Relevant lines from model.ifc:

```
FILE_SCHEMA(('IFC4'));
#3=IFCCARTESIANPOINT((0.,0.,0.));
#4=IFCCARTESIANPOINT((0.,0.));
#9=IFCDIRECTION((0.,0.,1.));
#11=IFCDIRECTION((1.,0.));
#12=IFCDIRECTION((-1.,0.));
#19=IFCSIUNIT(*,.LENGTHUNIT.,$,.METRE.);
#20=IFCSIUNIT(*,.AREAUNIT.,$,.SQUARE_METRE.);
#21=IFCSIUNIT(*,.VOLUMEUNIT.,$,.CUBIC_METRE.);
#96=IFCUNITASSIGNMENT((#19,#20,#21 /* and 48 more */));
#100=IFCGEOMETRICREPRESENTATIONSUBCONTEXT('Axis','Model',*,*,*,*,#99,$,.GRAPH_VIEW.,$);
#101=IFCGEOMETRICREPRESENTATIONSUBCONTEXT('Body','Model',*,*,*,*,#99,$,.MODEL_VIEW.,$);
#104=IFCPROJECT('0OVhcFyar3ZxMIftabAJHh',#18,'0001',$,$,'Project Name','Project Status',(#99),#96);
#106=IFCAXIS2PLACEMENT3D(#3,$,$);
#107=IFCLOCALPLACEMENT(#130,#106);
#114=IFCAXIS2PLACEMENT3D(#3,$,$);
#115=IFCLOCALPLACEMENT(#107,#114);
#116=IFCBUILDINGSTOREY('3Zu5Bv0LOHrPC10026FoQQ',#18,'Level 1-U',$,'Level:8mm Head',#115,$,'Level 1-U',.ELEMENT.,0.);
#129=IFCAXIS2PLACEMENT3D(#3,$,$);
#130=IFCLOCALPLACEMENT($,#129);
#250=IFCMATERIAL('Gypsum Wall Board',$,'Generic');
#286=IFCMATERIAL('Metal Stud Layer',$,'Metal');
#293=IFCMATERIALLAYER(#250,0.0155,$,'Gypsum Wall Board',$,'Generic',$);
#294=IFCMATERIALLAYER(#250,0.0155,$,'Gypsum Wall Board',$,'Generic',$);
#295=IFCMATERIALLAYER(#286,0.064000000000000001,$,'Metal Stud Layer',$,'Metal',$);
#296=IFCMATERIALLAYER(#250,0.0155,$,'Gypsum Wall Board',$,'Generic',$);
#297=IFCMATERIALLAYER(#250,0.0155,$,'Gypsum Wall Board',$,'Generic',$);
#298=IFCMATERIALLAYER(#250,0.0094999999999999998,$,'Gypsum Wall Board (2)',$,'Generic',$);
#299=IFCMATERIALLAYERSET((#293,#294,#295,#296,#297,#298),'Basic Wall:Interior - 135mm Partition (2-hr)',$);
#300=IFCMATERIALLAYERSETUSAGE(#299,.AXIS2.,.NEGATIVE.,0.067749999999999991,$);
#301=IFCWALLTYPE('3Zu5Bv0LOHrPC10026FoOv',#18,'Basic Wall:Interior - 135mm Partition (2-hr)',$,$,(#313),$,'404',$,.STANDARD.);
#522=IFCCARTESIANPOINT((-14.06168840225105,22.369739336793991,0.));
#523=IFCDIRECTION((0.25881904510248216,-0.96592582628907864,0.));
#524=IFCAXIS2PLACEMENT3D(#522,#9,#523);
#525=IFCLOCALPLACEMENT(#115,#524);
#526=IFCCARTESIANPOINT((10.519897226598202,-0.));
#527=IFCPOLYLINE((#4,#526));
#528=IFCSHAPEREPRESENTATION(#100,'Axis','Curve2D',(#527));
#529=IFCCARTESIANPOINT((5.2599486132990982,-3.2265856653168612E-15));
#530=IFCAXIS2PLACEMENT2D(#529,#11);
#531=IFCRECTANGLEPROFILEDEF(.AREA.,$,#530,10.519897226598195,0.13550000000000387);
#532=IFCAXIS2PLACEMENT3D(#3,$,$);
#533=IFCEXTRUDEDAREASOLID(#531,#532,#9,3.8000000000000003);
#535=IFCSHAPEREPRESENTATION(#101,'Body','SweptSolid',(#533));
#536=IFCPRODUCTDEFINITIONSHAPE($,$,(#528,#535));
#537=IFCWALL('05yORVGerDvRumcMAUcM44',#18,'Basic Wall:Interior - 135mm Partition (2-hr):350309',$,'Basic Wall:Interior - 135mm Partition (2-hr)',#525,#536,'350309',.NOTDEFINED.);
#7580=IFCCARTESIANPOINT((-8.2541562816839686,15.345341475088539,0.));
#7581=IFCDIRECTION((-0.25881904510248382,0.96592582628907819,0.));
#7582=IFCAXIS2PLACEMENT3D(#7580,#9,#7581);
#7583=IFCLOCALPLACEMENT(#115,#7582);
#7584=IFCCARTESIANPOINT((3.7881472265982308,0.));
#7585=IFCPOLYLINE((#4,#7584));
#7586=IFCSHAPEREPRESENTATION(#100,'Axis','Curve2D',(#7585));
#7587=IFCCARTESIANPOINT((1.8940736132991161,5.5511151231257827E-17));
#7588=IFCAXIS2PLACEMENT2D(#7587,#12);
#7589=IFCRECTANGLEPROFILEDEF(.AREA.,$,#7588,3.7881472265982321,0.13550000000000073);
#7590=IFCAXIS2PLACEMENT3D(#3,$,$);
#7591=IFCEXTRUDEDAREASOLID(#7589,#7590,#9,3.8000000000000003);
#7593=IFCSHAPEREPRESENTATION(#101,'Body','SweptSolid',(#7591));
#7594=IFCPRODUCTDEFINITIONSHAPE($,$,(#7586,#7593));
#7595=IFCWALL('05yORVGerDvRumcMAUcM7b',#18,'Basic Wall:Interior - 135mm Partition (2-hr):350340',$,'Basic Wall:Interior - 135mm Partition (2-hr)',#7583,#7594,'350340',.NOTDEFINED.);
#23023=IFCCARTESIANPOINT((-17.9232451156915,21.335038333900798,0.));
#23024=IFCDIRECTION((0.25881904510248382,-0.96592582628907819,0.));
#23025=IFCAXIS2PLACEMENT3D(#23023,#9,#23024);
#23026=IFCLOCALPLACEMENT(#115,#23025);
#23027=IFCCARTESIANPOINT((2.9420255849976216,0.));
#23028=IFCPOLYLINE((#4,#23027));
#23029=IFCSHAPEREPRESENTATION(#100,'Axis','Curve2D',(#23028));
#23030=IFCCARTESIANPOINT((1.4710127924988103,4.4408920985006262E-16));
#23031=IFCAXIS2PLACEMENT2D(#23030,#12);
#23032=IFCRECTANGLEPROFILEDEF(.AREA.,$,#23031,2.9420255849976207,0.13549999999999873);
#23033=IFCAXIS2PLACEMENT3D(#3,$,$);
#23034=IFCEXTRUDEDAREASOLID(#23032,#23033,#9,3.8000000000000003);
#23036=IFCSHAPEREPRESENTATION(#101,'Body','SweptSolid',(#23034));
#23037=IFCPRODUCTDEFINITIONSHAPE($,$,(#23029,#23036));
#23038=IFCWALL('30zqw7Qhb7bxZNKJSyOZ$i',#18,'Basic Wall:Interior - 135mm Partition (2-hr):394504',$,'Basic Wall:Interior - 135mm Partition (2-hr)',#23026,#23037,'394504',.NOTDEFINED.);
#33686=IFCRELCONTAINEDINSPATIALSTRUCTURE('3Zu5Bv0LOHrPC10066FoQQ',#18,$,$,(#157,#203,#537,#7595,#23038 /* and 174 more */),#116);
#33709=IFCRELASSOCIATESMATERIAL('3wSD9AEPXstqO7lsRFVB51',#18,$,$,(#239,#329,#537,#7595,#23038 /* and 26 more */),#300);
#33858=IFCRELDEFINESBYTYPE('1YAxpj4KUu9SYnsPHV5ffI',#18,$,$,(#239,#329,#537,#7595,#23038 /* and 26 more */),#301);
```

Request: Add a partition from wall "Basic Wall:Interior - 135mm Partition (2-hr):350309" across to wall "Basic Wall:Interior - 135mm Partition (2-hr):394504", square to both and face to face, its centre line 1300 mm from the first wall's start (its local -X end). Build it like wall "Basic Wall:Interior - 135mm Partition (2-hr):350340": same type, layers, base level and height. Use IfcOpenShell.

```python
import numpy as np
import ifcopenshell
import ifcopenshell.api.geometry
import ifcopenshell.api.material
import ifcopenshell.api.pset
import ifcopenshell.api.root
import ifcopenshell.api.spatial
import ifcopenshell.api.type
import ifcopenshell.geom
import ifcopenshell.util.element
import ifcopenshell.util.placement
import ifcopenshell.util.representation
import ifcopenshell.util.shape
import ifcopenshell.util.unit

model = ifcopenshell.open("model.ifc")
unit_scale = ifcopenshell.util.unit.calculate_unit_scale(model)
settings = ifcopenshell.geom.settings()
settings.set("use-world-coords", True)

start_wall = model.by_guid("05yORVGerDvRumcMAUcM44")
end_wall = model.by_guid("30zqw7Qhb7bxZNKJSyOZ$i")
like = model.by_guid("05yORVGerDvRumcMAUcM7b")
matrix = ifcopenshell.util.placement.get_local_placement(start_wall.ObjectPlacement)
matrix[:3, 3] *= unit_scale


def extent(element):
    """Bounding box in the first wall's axes, in metres."""
    shape = ifcopenshell.geom.create_shape(settings, element)
    points = (ifcopenshell.util.shape.get_vertices(shape.geometry) - matrix[:3, 3]) @ matrix[:3, :3]
    return points.min(axis=0), points.max(axis=0)


y_start = extent(start_wall)[0][1]
y_end = extent(end_wall)[1][1]
like_min, like_max = extent(like)
length, height = float(abs(y_end - y_start)), float(like_max[2] - like_min[2])
layer_set = ifcopenshell.util.element.get_material(like, should_skip_usage=True)
thickness = sum(layer.LayerThickness for layer in layer_set.MaterialLayers) * unit_scale

wall = ifcopenshell.api.root.create_entity(model, ifc_class="IfcWall", name="New partition")
storey = ifcopenshell.util.element.get_container(like)
ifcopenshell.api.spatial.assign_container(model, products=[wall], relating_structure=storey)
ifcopenshell.api.type.assign_type(
    model, related_objects=[wall], relating_type=ifcopenshell.util.element.get_type(like), should_map_representations=False
)
rel = ifcopenshell.api.material.assign_material(
    model, products=[wall], type="IfcMaterialLayerSetUsage", material=layer_set
)
rel.RelatingMaterial.OffsetFromReferenceLine = -thickness / 2 / unit_scale
pset = ifcopenshell.api.pset.add_pset(model, product=wall, name="Pset_WallCommon")
ifcopenshell.api.pset.edit_pset(model, pset=pset, properties={"IsExternal": False, "LoadBearing": False})

# The axis runs down the middle of the wall.
axis = ifcopenshell.api.geometry.add_axis_representation(
    model, context=ifcopenshell.util.representation.get_context(model, "Model", "Axis"), axis=[(0.0, 0.0), (length, 0.0)]
)
body = ifcopenshell.api.geometry.add_wall_representation(
    model,
    context=ifcopenshell.util.representation.get_context(model, "Model", "Body", "MODEL_VIEW"),
    length=length,
    height=height,
    thickness=thickness,
    offset=-thickness / 2,
)
for representation in (axis, body):
    ifcopenshell.api.geometry.assign_representation(model, product=wall, representation=representation)

placement = matrix @ ifcopenshell.util.placement.rotation(-90, "Z")
placement[:, 3] = matrix @ np.array([extent(start_wall)[0][0] + 1.3, y_start, like_min[2], 1.0])
ifcopenshell.api.geometry.edit_object_placement(model, product=wall, matrix=placement)

print(f"partition {length:.3f} m long, {height:.3f} m high, {thickness:.3f} m thick")

model.write("model_edited.ifc")
```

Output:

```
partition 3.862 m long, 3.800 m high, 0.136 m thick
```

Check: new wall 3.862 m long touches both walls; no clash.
